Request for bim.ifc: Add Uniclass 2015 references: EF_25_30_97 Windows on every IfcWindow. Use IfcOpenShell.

First a look at what the model holds.

```python
import ifcopenshell

model = ifcopenshell.open("bim.ifc")
print(model.schema)
print("classifications:", [c.Name for c in model.by_type("IfcClassification")])
for ifc_class in ("IfcDoor", "IfcRoof", "IfcStair", "IfcWall", "IfcWindow"):
    print(ifc_class, len(model.by_type(ifc_class)))
```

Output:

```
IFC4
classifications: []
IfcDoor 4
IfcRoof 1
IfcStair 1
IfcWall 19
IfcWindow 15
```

```python
import ifcopenshell
import ifcopenshell.api.classification

model = ifcopenshell.open("bim.ifc")

system = ifcopenshell.api.classification.add_classification(model, classification="Uniclass 2015")

codes = {
    "IfcWindow": ("EF_25_30_97", "Windows"),
}
for ifc_class, (code, name) in codes.items():
    products = model.by_type(ifc_class)
    ifcopenshell.api.classification.add_reference(
        model, products=products, classification=system, identification=code, name=name
    )
    print(code, len(products))

model.write("bim_edited.ifc")
```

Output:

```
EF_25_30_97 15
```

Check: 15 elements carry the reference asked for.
